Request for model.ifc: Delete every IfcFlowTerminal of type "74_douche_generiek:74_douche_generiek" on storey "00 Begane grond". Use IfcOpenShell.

First a look at what the model holds.

```python
import ifcopenshell
import ifcopenshell.util.element

model = ifcopenshell.open("model.ifc")
print(model.schema)
storey = next(s for s in model.by_type("IfcBuildingStorey") if s.Name == "00 Begane grond")
terminals = [e for e in ifcopenshell.util.element.get_decomposition(storey) if e.is_a("IfcFlowTerminal")]
seen = {}
for e in terminals:
    element_type = ifcopenshell.util.element.get_type(e)
    name = element_type.Name if element_type not in (None, e) else None
    seen[name] = seen.get(name, 0) + 1
for name, count in sorted(seen.items(), key=str):
    print(count, "x", name)
```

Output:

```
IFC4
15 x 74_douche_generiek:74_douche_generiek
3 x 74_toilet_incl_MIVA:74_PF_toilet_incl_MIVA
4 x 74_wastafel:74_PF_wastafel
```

```python
import ifcopenshell
import ifcopenshell.api.root
import ifcopenshell.util.element

model = ifcopenshell.open("model.ifc")

storey = next(s for s in model.by_type("IfcBuildingStorey") if s.Name == "00 Begane grond")
terminals = [e for e in ifcopenshell.util.element.get_decomposition(storey) if e.is_a("IfcFlowTerminal")]
targets = [e for e in terminals if (t := ifcopenshell.util.element.get_type(e)) not in (None, e) and t.Name == "74_douche_generiek:74_douche_generiek"]

for e in targets:
    ifcopenshell.api.root.remove_product(model, product=e)
print(len(targets), "removed")

model.write("model-out.ifc")
```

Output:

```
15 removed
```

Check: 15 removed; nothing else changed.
